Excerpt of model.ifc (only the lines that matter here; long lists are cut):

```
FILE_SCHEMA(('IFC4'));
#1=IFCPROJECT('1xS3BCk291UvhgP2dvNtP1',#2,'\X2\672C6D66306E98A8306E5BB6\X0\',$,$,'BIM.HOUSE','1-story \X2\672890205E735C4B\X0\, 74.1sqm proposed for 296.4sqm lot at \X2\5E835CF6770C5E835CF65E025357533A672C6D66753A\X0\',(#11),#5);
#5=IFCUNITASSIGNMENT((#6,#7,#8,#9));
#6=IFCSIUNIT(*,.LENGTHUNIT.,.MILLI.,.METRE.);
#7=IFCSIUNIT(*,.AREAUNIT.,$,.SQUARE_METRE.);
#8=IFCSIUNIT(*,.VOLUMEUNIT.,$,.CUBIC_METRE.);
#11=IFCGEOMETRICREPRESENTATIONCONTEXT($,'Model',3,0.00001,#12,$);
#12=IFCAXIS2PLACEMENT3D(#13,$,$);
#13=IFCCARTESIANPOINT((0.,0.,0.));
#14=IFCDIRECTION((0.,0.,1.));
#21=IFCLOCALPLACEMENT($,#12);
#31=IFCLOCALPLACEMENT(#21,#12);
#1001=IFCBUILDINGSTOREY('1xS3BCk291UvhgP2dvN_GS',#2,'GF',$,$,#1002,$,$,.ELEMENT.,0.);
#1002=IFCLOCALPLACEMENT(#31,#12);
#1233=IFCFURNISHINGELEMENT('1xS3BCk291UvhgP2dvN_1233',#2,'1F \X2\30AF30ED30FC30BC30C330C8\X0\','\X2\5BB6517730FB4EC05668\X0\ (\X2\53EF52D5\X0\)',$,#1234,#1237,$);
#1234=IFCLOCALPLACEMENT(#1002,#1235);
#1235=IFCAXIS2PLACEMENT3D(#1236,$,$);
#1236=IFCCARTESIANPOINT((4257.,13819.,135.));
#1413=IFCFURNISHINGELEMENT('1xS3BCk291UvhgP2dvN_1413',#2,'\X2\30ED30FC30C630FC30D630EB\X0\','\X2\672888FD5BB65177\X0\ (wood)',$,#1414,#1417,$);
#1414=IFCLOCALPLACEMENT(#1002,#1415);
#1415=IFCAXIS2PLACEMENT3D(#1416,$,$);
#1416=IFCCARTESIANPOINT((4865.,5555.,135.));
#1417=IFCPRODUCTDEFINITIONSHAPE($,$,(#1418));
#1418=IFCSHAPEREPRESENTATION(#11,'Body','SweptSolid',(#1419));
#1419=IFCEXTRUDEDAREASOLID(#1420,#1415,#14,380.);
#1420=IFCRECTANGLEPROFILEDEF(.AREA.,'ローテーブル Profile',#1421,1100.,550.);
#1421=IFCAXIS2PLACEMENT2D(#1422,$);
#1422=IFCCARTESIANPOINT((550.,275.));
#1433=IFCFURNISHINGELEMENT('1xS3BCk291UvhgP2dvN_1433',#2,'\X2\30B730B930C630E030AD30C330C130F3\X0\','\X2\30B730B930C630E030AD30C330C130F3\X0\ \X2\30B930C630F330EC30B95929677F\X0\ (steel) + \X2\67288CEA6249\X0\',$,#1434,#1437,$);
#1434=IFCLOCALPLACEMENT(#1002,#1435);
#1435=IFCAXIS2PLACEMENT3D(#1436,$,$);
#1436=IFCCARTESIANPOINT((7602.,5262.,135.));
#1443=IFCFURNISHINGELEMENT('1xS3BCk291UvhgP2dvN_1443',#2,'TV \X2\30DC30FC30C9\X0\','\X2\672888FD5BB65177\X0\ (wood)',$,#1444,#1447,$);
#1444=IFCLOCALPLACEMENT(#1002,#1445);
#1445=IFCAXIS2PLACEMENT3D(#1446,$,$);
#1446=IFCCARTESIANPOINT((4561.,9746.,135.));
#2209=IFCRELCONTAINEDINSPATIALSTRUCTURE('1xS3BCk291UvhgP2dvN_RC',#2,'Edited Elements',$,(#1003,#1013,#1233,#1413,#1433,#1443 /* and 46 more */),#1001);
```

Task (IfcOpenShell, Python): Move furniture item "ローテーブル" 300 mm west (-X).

```python
import ifcopenshell
import ifcopenshell.api.geometry
import ifcopenshell.util.placement
import ifcopenshell.util.unit

model = ifcopenshell.open("model.ifc")
unit_scale = ifcopenshell.util.unit.calculate_unit_scale(model)

item = model.by_id(1413)
matrix = ifcopenshell.util.placement.get_local_placement(item.ObjectPlacement)
matrix[0, 3] -= 0.3 / unit_scale
ifcopenshell.api.geometry.edit_object_placement(model, product=item, matrix=matrix, is_si=False)

print(ifcopenshell.util.placement.get_local_placement(item.ObjectPlacement).round(3) + 0.0)

model.write("model_edited.ifc")
```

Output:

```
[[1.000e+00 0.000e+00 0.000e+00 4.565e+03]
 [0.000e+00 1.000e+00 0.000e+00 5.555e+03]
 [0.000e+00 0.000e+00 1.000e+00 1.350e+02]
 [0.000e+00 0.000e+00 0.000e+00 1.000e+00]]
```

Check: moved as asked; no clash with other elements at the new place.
